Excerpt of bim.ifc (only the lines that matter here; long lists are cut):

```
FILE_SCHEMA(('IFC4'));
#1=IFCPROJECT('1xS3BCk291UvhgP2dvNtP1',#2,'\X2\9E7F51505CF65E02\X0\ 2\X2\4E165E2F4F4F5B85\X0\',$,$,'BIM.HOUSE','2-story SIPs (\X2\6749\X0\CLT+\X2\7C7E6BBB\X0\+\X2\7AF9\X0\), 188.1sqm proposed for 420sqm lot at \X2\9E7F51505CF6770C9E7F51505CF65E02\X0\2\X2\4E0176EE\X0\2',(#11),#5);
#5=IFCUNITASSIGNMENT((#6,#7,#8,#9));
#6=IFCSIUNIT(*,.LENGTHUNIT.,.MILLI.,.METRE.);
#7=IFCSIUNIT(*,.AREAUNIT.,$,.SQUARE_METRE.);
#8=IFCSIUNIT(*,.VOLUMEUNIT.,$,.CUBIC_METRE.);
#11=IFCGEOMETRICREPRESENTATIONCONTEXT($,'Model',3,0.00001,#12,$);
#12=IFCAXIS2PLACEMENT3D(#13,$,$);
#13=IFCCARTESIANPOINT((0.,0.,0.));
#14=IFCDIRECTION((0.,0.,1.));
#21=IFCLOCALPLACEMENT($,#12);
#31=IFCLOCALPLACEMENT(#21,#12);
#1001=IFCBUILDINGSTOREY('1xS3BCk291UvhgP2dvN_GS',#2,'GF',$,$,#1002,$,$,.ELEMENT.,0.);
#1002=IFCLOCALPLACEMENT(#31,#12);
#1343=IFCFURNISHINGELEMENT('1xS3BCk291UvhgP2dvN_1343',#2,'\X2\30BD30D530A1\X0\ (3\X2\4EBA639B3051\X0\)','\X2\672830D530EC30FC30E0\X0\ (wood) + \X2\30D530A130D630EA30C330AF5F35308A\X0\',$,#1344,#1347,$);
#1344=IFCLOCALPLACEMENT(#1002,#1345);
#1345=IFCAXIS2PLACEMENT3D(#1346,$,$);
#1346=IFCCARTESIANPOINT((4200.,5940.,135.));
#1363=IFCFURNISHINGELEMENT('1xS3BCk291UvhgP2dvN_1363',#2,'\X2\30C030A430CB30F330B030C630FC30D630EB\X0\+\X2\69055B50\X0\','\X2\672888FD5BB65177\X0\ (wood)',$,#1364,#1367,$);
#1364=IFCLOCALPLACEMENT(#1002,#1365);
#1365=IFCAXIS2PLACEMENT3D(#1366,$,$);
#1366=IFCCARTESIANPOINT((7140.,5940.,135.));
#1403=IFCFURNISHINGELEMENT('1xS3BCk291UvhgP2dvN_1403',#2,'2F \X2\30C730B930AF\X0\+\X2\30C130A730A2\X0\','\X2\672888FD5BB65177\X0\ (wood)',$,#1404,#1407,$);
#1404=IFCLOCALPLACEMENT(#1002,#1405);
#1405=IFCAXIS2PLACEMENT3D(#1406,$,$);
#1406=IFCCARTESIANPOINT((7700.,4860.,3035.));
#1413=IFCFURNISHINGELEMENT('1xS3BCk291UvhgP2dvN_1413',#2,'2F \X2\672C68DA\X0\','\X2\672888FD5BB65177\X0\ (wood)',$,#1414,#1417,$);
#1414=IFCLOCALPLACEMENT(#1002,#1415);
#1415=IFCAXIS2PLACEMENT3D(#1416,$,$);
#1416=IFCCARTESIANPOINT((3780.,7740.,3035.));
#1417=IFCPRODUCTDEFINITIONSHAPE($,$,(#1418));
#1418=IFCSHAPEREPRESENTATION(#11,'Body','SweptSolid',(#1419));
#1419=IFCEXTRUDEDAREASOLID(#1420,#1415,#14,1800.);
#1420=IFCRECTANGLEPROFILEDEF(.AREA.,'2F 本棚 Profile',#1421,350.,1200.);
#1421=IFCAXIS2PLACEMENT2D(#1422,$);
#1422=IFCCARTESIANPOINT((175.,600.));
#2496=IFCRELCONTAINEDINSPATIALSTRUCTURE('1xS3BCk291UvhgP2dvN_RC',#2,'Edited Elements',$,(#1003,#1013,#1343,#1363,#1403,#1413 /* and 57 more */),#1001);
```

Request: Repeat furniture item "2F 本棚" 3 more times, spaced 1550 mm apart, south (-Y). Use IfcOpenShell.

```python
import numpy as np
import ifcopenshell
import ifcopenshell.api.geometry
import ifcopenshell.api.root
import ifcopenshell.util.element
import ifcopenshell.util.placement
import ifcopenshell.util.unit

model = ifcopenshell.open("bim.ifc")
unit_scale = ifcopenshell.util.unit.calculate_unit_scale(model)


def reuse_history(source, copy):
    """copy_class also copies each property set's owner history, people and application; keep the originals."""
    for rel in copy.IsDefinedBy:
        if rel.is_a("IfcRelDefinesByProperties") and (history := rel.RelatingPropertyDefinition.OwnerHistory):
            rel.RelatingPropertyDefinition.OwnerHistory = source.OwnerHistory
            ifcopenshell.util.element.remove_deep2(model, history)


source = model.by_id(1413)
base = ifcopenshell.util.placement.get_local_placement(source.ObjectPlacement)
step = np.array([0.0, -1.0, 0.0]) * 1.55 / unit_scale

for i in range(1, 4):
    copy = ifcopenshell.api.root.copy_class(model, product=source)
    copy.Representation = ifcopenshell.util.element.copy_deep(
        model, source.Representation, exclude=["IfcGeometricRepresentationContext", "IfcRepresentationMap"]
    )
    reuse_history(source, copy)
    matrix = base.copy()
    matrix[:3, 3] += i * step
    print("added at", matrix[:3, 3].round(3) + 0.0)
    ifcopenshell.api.geometry.edit_object_placement(model, product=copy, matrix=matrix, is_si=False)

model.write("bim-out.ifc")
```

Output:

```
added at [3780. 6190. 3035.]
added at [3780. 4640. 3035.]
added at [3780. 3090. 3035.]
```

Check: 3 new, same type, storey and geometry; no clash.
